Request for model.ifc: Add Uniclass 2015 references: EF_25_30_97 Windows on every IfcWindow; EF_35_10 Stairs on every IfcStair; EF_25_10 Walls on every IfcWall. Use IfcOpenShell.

First a look at what the model holds.

```python
import ifcopenshell

model = ifcopenshell.open("model.ifc")
print(model.schema)
print("classifications:", [c.Name for c in model.by_type("IfcClassification")])
for ifc_class in ("IfcDoor", "IfcRoof", "IfcStair", "IfcWall", "IfcWindow"):
    print(ifc_class, len(model.by_type(ifc_class)))
```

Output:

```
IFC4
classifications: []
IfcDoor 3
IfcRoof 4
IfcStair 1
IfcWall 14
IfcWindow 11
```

```python
import ifcopenshell
import ifcopenshell.api.classification

model = ifcopenshell.open("model.ifc")

system = ifcopenshell.api.classification.add_classification(model, classification="Uniclass 2015")

codes = {
    "IfcWindow": ("EF_25_30_97", "Windows"),
    "IfcStair": ("EF_35_10", "Stairs"),
    "IfcWall": ("EF_25_10", "Walls"),
}
for ifc_class, (code, name) in codes.items():
    products = model.by_type(ifc_class)
    ifcopenshell.api.classification.add_reference(
        model, products=products, classification=system, identification=code, name=name
    )
    print(code, len(products))

model.write("model_edited.ifc")
```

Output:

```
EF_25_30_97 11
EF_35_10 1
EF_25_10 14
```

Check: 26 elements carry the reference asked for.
